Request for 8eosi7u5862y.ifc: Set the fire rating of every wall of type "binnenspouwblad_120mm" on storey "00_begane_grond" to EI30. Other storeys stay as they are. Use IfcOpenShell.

First a look at what the model holds.

```python
import ifcopenshell
import ifcopenshell.util.element

model = ifcopenshell.open("8eosi7u5862y.ifc")
print(model.schema)
storey = next(s for s in model.by_type("IfcBuildingStorey") if s.Name == "00_begane_grond")
walls = [e for e in ifcopenshell.util.element.get_decomposition(storey) if e.is_a("IfcWall")]
seen = {}
for e in walls:
    element_type = ifcopenshell.util.element.get_type(e)
    key = (element_type.Name if element_type != e and element_type else None, ifcopenshell.util.element.get_pset(e, "Pset_WallCommon", "FireRating"))
    seen[key] = seen.get(key, 0) + 1
for (name, value), count in sorted(seen.items(), key=str):
    print(count, "x", name, "|", value)
```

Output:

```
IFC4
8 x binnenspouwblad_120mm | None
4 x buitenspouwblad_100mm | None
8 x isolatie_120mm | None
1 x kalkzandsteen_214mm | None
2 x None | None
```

```python
import ifcopenshell
import ifcopenshell.api.pset
import ifcopenshell.util.element

model = ifcopenshell.open("8eosi7u5862y.ifc")

storey = next(s for s in model.by_type("IfcBuildingStorey") if s.Name == "00_begane_grond")
walls = [e for e in ifcopenshell.util.element.get_decomposition(storey) if e.is_a("IfcWall")]

count = 0
for e in walls:
    element_type = ifcopenshell.util.element.get_type(e)
    if element_type in (None, e) or element_type.Name != "binnenspouwblad_120mm":
        continue
    # add_pset returns the element's existing set when there is one.
    pset = ifcopenshell.api.pset.add_pset(model, product=e, name="Pset_WallCommon")
    ifcopenshell.api.pset.edit_pset(model, pset=pset, properties={"FireRating": "EI30"})
    count += 1

print(count, "walls updated")

model.write("8eosi7u5862y_edited.ifc")
```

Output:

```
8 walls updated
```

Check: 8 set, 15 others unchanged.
